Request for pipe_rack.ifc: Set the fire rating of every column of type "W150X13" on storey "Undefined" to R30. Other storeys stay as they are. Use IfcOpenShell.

First a look at what the model holds.

```python
import ifcopenshell
import ifcopenshell.util.element

model = ifcopenshell.open("pipe_rack.ifc")
print(model.schema)
storey = next(s for s in model.by_type("IfcBuildingStorey") if s.Name == "Undefined")
columns = [e for e in ifcopenshell.util.element.get_decomposition(storey) if e.is_a("IfcColumn")]
seen = {}
for e in columns:
    element_type = ifcopenshell.util.element.get_type(e)
    key = (element_type.Name if element_type != e and element_type else None, ifcopenshell.util.element.get_pset(e, "Pset_ColumnCommon", "FireRating"))
    seen[key] = seen.get(key, 0) + 1
for (name, value), count in sorted(seen.items(), key=str):
    print(count, "x", name, "|", value)
```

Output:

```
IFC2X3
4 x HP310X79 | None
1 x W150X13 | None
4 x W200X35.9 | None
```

```python
import ifcopenshell
import ifcopenshell.api.pset
import ifcopenshell.util.element

model = ifcopenshell.open("pipe_rack.ifc")

storey = next(s for s in model.by_type("IfcBuildingStorey") if s.Name == "Undefined")
columns = [e for e in ifcopenshell.util.element.get_decomposition(storey) if e.is_a("IfcColumn")]

count = 0
for e in columns:
    element_type = ifcopenshell.util.element.get_type(e)
    if element_type in (None, e) or element_type.Name != "W150X13":
        continue
    # add_pset returns the element's existing set when there is one.
    pset = ifcopenshell.api.pset.add_pset(model, product=e, name="Pset_ColumnCommon")
    ifcopenshell.api.pset.edit_pset(model, pset=pset, properties={"FireRating": "R30"})
    count += 1

print(count, "columns updated")

model.write("pipe_rack_v2.ifc")
```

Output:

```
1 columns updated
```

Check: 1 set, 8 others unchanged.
